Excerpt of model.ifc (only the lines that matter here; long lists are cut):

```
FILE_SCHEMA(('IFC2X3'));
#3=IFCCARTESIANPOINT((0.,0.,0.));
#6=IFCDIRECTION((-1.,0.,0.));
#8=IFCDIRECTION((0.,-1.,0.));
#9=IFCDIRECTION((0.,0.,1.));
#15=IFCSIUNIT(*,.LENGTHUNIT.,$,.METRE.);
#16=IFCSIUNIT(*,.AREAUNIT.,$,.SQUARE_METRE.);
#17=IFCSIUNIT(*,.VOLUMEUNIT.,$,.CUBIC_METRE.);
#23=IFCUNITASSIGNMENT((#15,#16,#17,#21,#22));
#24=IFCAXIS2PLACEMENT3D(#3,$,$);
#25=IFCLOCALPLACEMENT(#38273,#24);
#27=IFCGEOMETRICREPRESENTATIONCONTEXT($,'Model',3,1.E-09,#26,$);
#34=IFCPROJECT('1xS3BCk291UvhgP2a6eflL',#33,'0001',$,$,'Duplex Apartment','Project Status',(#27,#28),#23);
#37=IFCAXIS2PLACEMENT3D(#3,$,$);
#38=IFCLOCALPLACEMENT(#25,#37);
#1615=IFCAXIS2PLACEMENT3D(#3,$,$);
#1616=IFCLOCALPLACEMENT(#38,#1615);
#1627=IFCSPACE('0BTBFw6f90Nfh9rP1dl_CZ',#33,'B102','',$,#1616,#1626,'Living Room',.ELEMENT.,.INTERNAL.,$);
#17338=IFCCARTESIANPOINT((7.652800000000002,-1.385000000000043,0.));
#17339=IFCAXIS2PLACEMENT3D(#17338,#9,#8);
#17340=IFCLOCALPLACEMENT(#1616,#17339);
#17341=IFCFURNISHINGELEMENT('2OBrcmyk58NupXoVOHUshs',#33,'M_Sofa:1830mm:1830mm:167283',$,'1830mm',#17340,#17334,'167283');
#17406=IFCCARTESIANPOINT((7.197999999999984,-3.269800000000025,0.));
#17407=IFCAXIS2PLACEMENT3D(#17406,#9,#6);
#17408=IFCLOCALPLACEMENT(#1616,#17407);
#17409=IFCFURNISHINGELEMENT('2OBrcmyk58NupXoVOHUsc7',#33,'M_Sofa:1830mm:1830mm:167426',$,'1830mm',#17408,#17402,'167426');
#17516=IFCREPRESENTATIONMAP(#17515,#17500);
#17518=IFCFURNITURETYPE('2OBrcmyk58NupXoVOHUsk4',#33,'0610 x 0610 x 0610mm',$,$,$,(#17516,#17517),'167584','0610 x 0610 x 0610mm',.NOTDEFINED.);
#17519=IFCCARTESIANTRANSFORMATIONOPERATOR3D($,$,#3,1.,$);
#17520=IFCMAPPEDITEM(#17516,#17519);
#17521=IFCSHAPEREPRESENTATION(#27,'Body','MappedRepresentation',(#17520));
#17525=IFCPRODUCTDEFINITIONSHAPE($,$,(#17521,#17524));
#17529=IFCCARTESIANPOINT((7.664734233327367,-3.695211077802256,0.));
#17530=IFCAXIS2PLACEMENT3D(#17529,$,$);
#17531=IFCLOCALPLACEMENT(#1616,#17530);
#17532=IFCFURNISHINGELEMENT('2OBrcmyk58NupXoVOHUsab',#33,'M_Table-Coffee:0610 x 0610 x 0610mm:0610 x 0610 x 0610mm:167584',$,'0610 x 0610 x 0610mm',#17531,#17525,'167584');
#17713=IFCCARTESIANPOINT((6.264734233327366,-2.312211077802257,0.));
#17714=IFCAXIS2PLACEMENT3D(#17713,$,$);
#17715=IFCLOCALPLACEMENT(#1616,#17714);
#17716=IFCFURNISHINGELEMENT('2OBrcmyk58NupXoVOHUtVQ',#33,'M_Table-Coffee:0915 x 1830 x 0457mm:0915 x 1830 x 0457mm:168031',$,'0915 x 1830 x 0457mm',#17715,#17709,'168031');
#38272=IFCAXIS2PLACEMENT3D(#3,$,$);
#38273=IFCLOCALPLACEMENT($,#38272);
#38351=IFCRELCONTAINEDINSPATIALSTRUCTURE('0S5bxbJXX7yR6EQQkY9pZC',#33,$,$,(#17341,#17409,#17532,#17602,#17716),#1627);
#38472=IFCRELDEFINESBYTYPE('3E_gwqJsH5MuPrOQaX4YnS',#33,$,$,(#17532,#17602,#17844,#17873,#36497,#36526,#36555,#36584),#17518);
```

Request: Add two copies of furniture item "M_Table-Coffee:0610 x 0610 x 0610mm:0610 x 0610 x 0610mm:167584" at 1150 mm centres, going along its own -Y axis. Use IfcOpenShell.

```python
import ifcopenshell
import ifcopenshell.api.geometry
import ifcopenshell.api.root
import ifcopenshell.util.element
import ifcopenshell.util.placement
import ifcopenshell.util.unit

model = ifcopenshell.open("model.ifc")
unit_scale = ifcopenshell.util.unit.calculate_unit_scale(model)


def reuse_history(source, copy):
    """copy_class also copies each property set's owner history, people and application; keep the originals."""
    for rel in copy.IsDefinedBy:
        if rel.is_a("IfcRelDefinesByProperties") and (history := rel.RelatingPropertyDefinition.OwnerHistory):
            rel.RelatingPropertyDefinition.OwnerHistory = source.OwnerHistory
            ifcopenshell.util.element.remove_deep2(model, history)


source = model.by_id(17532)
base = ifcopenshell.util.placement.get_local_placement(source.ObjectPlacement)
step = -base[:3, 1] * 1.15 / unit_scale

for i in range(1, 3):
    copy = ifcopenshell.api.root.copy_class(model, product=source)
    copy.Representation = ifcopenshell.util.element.copy_deep(
        model, source.Representation, exclude=["IfcGeometricRepresentationContext", "IfcRepresentationMap"]
    )
    copy.Name = "M_Table-Coffee:0610 x 0610 x 0610mm:0610 x 0610 x 0610mm"
    copy.Tag = None
    reuse_history(source, copy)
    matrix = base.copy()
    matrix[:3, 3] += i * step
    print("added at", matrix[:3, 3].round(3) + 0.0)
    ifcopenshell.api.geometry.edit_object_placement(model, product=copy, matrix=matrix, is_si=False)

model.write("model_v2.ifc")
```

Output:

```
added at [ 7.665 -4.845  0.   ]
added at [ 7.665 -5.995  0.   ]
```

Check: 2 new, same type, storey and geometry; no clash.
